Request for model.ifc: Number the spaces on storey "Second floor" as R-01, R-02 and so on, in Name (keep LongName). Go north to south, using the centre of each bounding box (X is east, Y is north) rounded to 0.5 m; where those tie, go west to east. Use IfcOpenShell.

First a look at what the model holds.

```python
import ifcopenshell
import ifcopenshell.util.element
import ifcopenshell.util.placement

model = ifcopenshell.open("model.ifc")
print(model.schema)
storey = next(s for s in model.by_type("IfcBuildingStorey") if s.Name == "Second floor")
spaces = [e for e in ifcopenshell.util.element.get_decomposition(storey) if e.is_a("IfcSpace")]
for e in sorted(spaces, key=lambda e: e.id()):
    origin = ifcopenshell.util.placement.get_local_placement(e.ObjectPlacement)[:3, 3]
    print(e.id(), e.Name, e.LongName, origin.round(2) + 0.0, sep=" | ")
```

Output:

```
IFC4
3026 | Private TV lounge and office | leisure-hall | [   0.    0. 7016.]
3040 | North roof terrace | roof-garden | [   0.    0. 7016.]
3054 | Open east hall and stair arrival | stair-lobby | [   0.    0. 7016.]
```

```python
import ifcopenshell
import ifcopenshell.geom
import ifcopenshell.util.element
import ifcopenshell.util.shape

model = ifcopenshell.open("model.ifc")
settings = ifcopenshell.geom.settings()
settings.set("use-world-coords", True)


def centre(element):
    shape = ifcopenshell.geom.create_shape(settings, element)
    return ifcopenshell.util.shape.get_bbox_centroid(shape.geometry)


storey = next(s for s in model.by_type("IfcBuildingStorey") if s.Name == "Second floor")
spaces = [e for e in ifcopenshell.util.element.get_decomposition(storey) if e.is_a("IfcSpace")]

# Insertion points can sit at a corner or the storey origin, so sort by the geometry (in metres).
centres = {e: centre(e) for e in spaces}
spaces.sort(key=lambda e: (-round(centres[e][1] / 0.5), centres[e][0]))

for i, e in enumerate(spaces, start=1):
    number = f"R-{i:02d}"
    e.Name = number
    print(e.id(), number)

model.write("model_rev.ifc")
```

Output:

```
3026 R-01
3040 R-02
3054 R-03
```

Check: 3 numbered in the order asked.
